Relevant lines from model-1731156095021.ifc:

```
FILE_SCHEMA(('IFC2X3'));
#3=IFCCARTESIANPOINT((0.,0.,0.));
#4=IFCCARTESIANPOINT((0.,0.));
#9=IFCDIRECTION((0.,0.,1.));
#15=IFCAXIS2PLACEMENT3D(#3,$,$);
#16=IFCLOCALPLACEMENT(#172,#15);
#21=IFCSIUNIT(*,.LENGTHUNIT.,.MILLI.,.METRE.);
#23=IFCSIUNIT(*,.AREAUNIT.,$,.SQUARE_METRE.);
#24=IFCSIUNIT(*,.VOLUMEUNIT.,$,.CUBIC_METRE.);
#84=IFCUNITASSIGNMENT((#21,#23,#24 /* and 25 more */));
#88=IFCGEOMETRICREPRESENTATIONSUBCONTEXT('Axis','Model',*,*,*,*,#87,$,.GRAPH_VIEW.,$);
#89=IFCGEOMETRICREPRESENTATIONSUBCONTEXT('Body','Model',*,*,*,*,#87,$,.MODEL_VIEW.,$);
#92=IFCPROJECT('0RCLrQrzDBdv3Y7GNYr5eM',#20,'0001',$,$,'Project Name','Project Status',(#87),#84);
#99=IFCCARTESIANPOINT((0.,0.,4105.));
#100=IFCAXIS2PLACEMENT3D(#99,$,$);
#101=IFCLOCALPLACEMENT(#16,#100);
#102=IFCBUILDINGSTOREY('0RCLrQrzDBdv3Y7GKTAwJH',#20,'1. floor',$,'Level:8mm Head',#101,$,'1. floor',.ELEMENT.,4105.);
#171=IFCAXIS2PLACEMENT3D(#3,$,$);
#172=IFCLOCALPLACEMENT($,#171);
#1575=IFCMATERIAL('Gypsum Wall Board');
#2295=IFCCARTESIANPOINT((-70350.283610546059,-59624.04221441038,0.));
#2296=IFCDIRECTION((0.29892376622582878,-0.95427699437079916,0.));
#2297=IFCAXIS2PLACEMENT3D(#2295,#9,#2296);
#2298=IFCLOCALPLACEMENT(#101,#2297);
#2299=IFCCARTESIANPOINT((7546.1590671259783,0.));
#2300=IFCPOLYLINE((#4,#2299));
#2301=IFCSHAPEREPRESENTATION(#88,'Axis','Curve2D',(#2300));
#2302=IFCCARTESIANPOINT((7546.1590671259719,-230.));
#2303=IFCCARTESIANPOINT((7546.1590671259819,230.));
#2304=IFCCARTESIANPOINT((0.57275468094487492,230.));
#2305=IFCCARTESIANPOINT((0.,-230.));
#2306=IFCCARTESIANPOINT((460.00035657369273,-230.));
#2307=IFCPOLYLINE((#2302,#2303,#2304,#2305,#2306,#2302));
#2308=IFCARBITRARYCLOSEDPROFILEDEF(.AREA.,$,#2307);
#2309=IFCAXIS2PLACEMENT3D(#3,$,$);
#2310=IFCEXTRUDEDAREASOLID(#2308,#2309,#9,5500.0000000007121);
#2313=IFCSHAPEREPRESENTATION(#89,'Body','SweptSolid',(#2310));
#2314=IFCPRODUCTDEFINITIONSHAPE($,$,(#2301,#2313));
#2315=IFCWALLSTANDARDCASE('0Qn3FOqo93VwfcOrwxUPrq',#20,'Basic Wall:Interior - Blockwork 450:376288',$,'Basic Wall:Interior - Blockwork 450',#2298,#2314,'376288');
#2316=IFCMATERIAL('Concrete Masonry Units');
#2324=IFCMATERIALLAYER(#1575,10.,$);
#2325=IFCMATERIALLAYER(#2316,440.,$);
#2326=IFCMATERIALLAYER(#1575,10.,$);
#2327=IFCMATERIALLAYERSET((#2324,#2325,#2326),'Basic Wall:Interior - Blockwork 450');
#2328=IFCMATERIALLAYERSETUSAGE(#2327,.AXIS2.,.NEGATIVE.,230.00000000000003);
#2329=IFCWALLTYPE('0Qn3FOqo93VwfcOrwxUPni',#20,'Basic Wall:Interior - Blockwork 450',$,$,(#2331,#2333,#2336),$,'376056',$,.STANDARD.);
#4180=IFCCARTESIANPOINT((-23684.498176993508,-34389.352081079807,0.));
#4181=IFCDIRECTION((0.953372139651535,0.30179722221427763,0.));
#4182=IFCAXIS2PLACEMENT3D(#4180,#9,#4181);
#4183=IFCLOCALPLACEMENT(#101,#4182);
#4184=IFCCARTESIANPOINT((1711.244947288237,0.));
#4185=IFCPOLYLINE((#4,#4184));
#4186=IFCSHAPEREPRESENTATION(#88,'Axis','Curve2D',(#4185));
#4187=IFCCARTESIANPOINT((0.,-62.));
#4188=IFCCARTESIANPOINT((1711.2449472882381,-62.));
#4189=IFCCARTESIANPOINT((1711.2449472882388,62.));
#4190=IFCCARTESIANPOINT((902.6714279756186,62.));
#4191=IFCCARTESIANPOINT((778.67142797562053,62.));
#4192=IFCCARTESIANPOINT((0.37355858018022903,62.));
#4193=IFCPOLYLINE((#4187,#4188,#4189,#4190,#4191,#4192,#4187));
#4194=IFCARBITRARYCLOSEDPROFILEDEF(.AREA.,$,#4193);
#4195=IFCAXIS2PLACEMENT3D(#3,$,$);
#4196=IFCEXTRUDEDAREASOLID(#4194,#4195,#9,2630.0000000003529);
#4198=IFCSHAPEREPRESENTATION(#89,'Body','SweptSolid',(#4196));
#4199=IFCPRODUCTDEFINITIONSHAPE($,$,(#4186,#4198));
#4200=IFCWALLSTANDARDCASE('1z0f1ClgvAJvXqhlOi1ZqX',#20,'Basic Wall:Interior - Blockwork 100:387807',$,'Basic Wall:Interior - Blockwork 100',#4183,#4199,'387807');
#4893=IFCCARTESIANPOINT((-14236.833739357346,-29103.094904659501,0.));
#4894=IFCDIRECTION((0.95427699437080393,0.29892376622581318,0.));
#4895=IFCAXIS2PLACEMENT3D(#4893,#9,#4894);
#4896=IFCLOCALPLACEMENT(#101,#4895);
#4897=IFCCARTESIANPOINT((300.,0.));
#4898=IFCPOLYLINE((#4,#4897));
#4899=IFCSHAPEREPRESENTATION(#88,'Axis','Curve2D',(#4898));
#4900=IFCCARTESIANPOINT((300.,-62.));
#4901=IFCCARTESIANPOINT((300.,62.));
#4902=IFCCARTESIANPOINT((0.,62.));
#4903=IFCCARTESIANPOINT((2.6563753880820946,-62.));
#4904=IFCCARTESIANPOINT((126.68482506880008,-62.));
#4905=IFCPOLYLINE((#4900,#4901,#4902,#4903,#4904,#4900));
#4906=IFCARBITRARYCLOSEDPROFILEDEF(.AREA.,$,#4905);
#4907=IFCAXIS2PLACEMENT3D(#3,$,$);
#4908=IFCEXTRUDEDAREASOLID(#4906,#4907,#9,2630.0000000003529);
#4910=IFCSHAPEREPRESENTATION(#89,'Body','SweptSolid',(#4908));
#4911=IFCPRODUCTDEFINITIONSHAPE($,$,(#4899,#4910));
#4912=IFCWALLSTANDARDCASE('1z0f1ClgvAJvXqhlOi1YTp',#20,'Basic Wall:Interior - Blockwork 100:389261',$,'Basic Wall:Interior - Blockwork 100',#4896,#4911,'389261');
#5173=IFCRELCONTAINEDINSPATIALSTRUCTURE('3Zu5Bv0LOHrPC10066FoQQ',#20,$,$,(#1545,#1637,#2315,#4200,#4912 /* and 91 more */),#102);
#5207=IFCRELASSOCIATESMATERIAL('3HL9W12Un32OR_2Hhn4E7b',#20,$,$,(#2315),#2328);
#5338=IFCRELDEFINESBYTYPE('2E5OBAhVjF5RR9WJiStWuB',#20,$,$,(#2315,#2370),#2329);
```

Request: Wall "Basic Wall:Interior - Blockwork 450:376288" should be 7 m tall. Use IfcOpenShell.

```python
import ifcopenshell
import ifcopenshell.geom
import ifcopenshell.util.representation
import ifcopenshell.util.shape
import ifcopenshell.util.unit

model = ifcopenshell.open("model-1731156095021.ifc")
unit_scale = ifcopenshell.util.unit.calculate_unit_scale(model)
settings = ifcopenshell.geom.settings()


def volume(element):
    """Net volume in cubic metres, openings subtracted."""
    shape = ifcopenshell.geom.create_shape(settings, element)
    return ifcopenshell.util.shape.get_volume(shape.geometry)


wall = model.by_guid("0Qn3FOqo93VwfcOrwxUPrq")
before = volume(wall)

body = ifcopenshell.util.representation.get_representation(wall, "Model", "Body")
solid = body.Items[0]
old_height = solid.Depth
solid.Depth = 7 / unit_scale
after = volume(wall)

print(f"height {old_height:g} -> {solid.Depth:g}, volume {before:.3f} -> {after:.3f} m3")

model.write("model-1731156095021-out.ifc")
```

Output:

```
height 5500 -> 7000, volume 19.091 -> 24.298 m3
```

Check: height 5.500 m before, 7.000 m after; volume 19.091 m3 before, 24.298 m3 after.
